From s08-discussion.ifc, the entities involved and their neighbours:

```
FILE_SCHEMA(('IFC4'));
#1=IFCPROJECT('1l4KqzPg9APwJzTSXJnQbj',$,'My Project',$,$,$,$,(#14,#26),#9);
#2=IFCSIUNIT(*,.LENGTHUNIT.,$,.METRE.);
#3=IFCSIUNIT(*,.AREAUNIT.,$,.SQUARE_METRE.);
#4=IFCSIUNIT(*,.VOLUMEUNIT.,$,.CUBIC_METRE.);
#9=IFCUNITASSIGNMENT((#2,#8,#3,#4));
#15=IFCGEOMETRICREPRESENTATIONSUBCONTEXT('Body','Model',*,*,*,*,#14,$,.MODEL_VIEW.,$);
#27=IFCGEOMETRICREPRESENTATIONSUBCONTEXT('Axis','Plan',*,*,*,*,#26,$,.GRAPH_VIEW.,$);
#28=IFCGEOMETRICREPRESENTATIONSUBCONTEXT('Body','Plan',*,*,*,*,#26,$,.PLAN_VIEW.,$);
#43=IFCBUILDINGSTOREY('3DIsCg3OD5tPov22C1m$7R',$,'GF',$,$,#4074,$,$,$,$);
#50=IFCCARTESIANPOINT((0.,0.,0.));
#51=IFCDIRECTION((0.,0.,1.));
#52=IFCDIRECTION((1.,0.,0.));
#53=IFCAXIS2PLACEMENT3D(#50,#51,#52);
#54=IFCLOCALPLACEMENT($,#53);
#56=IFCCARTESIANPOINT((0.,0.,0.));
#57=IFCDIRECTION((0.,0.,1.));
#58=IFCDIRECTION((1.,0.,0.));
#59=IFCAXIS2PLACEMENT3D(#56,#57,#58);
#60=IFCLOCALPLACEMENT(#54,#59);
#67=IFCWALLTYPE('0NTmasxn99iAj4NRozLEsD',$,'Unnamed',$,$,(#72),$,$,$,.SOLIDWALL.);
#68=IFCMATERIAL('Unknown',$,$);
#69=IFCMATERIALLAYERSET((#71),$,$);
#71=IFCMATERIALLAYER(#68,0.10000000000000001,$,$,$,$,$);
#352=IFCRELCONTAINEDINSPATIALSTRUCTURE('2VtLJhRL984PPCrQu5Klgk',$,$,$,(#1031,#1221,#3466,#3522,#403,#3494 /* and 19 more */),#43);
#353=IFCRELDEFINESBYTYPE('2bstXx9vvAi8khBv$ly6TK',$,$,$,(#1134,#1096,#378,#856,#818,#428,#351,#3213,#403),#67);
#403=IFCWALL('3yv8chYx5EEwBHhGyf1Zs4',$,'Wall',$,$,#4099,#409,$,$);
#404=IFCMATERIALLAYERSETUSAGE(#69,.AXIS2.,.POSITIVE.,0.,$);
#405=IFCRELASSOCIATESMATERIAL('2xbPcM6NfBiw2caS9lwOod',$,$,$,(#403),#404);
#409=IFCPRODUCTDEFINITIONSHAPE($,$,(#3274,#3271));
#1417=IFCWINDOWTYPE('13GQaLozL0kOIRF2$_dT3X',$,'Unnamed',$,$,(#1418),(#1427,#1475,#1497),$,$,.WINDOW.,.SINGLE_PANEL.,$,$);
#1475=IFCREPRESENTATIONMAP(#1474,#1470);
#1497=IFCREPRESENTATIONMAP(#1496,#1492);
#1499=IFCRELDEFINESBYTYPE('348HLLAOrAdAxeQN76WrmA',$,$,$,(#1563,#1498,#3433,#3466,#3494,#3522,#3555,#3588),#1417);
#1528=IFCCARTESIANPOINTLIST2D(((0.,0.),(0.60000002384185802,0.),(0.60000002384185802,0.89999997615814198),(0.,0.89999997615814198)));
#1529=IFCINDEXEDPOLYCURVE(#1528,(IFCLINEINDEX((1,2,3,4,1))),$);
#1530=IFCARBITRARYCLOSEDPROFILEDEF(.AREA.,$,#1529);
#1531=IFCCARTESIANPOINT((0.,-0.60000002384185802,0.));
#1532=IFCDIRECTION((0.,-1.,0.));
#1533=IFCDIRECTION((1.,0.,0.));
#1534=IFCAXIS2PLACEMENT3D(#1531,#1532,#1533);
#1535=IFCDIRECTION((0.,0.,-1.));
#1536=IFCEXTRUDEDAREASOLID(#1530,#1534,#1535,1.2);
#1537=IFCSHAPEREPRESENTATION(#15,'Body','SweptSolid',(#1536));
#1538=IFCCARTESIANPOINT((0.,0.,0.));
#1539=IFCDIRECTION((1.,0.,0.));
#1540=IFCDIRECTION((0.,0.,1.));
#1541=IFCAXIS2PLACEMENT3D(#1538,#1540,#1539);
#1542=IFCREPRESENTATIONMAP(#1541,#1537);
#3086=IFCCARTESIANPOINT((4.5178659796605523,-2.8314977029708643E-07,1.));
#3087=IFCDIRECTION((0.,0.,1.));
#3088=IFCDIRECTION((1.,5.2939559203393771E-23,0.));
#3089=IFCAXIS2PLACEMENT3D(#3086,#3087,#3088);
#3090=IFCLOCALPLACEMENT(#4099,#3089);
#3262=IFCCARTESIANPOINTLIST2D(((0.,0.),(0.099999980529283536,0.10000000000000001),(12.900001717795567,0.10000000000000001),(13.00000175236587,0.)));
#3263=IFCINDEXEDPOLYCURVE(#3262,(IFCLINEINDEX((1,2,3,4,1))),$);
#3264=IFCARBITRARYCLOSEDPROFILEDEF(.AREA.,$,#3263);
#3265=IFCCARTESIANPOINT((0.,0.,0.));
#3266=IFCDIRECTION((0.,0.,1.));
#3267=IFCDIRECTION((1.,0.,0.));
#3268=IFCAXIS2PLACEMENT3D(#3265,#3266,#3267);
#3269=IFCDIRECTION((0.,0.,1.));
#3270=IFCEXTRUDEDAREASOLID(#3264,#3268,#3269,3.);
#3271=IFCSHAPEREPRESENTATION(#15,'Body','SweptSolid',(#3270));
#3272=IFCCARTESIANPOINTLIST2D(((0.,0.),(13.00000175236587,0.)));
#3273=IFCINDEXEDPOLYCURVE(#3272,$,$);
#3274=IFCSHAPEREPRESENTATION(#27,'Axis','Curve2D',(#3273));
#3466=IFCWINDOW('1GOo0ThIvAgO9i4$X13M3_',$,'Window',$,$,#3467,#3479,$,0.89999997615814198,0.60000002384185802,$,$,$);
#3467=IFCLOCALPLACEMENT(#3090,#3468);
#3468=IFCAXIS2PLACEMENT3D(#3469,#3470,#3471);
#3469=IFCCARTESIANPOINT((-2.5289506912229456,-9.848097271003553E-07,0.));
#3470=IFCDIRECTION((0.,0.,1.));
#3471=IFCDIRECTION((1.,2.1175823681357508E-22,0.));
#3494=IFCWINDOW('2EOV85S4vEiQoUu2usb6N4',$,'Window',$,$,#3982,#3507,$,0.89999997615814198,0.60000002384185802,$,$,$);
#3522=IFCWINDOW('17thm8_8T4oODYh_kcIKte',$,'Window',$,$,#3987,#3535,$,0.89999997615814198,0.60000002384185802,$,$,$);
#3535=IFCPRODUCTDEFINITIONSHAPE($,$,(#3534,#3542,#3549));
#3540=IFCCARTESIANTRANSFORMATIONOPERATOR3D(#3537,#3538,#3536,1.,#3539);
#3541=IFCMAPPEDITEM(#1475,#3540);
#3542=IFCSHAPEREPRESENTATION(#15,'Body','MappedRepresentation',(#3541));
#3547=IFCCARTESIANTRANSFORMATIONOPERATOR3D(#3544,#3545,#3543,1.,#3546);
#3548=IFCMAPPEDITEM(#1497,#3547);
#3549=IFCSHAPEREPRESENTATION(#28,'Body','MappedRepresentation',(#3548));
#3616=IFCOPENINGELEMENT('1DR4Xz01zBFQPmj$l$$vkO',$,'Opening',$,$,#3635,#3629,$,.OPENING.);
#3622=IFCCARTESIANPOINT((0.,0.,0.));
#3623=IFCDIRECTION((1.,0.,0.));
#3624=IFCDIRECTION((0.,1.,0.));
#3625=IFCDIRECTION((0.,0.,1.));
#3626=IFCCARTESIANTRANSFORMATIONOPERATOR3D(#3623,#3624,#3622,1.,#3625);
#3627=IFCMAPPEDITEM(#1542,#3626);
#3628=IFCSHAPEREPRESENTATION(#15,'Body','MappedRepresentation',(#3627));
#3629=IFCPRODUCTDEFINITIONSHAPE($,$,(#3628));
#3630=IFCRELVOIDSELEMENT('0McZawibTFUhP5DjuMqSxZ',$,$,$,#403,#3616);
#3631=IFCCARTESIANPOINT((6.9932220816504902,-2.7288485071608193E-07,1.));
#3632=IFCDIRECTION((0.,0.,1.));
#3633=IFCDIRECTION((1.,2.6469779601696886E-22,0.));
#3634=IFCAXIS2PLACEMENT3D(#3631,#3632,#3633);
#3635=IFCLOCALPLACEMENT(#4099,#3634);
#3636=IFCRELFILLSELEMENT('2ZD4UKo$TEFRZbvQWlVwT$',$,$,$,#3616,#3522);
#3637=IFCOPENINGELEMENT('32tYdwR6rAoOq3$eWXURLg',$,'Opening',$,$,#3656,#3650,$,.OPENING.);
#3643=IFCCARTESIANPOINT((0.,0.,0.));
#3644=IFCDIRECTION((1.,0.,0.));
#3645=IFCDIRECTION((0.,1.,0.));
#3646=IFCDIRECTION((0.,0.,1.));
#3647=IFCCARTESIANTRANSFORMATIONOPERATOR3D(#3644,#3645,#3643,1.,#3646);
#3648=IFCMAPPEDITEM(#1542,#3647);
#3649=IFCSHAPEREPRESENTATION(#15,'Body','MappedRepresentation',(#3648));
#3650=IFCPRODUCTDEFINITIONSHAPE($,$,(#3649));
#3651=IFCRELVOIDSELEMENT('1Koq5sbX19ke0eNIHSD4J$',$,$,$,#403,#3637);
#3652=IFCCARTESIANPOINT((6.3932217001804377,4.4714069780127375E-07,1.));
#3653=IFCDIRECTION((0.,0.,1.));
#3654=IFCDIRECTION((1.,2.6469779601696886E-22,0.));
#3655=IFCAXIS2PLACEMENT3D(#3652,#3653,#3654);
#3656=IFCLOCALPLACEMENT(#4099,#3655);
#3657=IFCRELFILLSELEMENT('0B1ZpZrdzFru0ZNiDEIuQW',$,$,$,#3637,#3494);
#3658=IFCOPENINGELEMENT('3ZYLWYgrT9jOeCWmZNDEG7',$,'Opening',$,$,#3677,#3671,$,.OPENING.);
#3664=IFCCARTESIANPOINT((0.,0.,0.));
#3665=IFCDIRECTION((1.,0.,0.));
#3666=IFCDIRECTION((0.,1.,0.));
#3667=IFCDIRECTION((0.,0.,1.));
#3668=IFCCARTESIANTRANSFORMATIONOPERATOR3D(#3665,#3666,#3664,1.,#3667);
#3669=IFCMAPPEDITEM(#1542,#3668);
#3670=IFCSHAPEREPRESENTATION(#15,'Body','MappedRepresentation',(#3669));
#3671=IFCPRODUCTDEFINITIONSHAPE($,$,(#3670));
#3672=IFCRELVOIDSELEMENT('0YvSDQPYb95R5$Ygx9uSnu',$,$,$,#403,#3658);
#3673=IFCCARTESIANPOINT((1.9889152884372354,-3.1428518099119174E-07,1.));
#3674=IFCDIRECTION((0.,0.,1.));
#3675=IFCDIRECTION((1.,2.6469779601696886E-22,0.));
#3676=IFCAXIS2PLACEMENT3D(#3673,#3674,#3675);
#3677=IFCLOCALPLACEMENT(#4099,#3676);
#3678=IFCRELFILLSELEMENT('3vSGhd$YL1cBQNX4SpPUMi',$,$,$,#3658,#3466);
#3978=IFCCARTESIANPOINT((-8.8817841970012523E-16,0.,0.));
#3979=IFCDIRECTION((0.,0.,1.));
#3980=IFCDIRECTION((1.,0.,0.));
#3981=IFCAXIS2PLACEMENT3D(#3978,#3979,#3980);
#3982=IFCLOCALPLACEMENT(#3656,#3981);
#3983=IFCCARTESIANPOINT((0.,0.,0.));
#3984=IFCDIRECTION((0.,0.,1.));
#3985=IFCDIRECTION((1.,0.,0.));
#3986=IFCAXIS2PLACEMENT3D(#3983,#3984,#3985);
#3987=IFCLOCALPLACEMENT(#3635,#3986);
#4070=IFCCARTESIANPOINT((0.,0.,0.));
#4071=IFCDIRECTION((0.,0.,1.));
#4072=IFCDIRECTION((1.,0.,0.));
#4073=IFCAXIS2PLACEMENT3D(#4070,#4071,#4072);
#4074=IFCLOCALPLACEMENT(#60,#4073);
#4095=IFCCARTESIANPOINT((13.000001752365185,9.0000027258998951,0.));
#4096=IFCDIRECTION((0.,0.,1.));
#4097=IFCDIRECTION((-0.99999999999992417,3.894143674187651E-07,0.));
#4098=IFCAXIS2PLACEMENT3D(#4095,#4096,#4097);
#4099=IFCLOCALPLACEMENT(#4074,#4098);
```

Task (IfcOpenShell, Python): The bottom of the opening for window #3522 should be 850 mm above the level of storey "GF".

```python
import numpy as np
import ifcopenshell
import ifcopenshell.api.geometry
import ifcopenshell.geom
import ifcopenshell.util.element
import ifcopenshell.util.placement
import ifcopenshell.util.shape
import ifcopenshell.util.unit

model = ifcopenshell.open("s08-discussion.ifc")
unit_scale = ifcopenshell.util.unit.calculate_unit_scale(model)

window = model.by_guid("17thm8_8T4oODYh_kcIKte")
opening = window.FillsVoids[0].RelatingOpeningElement
storey = ifcopenshell.util.element.get_container(window, ifc_class="IfcBuildingStorey")
level = ifcopenshell.util.placement.get_local_placement(storey.ObjectPlacement)[2, 3]

# The opening's origin need not be at the sill, so measure its lowest point.
shape = ifcopenshell.geom.create_shape(ifcopenshell.geom.settings(), opening)
bottom = ifcopenshell.util.shape.get_shape_bottom_elevation(shape, shape.geometry) / unit_scale
dz = level + 0.85 - bottom

shift = np.array([0.0, 0.0, dz])
# The window is placed relative to its opening, so it follows when the opening moves.
matrix = ifcopenshell.util.placement.get_local_placement(opening.ObjectPlacement)
matrix[:3, 3] += shift
ifcopenshell.api.geometry.edit_object_placement(
    model, product=opening, matrix=matrix, is_si=False, should_transform_children=True
)

print(f"moved by {dz * unit_scale:+.3f} m")

model.write("s08-discussion_updated.ifc")
```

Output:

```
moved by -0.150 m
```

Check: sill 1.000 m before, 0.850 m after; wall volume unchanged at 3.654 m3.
